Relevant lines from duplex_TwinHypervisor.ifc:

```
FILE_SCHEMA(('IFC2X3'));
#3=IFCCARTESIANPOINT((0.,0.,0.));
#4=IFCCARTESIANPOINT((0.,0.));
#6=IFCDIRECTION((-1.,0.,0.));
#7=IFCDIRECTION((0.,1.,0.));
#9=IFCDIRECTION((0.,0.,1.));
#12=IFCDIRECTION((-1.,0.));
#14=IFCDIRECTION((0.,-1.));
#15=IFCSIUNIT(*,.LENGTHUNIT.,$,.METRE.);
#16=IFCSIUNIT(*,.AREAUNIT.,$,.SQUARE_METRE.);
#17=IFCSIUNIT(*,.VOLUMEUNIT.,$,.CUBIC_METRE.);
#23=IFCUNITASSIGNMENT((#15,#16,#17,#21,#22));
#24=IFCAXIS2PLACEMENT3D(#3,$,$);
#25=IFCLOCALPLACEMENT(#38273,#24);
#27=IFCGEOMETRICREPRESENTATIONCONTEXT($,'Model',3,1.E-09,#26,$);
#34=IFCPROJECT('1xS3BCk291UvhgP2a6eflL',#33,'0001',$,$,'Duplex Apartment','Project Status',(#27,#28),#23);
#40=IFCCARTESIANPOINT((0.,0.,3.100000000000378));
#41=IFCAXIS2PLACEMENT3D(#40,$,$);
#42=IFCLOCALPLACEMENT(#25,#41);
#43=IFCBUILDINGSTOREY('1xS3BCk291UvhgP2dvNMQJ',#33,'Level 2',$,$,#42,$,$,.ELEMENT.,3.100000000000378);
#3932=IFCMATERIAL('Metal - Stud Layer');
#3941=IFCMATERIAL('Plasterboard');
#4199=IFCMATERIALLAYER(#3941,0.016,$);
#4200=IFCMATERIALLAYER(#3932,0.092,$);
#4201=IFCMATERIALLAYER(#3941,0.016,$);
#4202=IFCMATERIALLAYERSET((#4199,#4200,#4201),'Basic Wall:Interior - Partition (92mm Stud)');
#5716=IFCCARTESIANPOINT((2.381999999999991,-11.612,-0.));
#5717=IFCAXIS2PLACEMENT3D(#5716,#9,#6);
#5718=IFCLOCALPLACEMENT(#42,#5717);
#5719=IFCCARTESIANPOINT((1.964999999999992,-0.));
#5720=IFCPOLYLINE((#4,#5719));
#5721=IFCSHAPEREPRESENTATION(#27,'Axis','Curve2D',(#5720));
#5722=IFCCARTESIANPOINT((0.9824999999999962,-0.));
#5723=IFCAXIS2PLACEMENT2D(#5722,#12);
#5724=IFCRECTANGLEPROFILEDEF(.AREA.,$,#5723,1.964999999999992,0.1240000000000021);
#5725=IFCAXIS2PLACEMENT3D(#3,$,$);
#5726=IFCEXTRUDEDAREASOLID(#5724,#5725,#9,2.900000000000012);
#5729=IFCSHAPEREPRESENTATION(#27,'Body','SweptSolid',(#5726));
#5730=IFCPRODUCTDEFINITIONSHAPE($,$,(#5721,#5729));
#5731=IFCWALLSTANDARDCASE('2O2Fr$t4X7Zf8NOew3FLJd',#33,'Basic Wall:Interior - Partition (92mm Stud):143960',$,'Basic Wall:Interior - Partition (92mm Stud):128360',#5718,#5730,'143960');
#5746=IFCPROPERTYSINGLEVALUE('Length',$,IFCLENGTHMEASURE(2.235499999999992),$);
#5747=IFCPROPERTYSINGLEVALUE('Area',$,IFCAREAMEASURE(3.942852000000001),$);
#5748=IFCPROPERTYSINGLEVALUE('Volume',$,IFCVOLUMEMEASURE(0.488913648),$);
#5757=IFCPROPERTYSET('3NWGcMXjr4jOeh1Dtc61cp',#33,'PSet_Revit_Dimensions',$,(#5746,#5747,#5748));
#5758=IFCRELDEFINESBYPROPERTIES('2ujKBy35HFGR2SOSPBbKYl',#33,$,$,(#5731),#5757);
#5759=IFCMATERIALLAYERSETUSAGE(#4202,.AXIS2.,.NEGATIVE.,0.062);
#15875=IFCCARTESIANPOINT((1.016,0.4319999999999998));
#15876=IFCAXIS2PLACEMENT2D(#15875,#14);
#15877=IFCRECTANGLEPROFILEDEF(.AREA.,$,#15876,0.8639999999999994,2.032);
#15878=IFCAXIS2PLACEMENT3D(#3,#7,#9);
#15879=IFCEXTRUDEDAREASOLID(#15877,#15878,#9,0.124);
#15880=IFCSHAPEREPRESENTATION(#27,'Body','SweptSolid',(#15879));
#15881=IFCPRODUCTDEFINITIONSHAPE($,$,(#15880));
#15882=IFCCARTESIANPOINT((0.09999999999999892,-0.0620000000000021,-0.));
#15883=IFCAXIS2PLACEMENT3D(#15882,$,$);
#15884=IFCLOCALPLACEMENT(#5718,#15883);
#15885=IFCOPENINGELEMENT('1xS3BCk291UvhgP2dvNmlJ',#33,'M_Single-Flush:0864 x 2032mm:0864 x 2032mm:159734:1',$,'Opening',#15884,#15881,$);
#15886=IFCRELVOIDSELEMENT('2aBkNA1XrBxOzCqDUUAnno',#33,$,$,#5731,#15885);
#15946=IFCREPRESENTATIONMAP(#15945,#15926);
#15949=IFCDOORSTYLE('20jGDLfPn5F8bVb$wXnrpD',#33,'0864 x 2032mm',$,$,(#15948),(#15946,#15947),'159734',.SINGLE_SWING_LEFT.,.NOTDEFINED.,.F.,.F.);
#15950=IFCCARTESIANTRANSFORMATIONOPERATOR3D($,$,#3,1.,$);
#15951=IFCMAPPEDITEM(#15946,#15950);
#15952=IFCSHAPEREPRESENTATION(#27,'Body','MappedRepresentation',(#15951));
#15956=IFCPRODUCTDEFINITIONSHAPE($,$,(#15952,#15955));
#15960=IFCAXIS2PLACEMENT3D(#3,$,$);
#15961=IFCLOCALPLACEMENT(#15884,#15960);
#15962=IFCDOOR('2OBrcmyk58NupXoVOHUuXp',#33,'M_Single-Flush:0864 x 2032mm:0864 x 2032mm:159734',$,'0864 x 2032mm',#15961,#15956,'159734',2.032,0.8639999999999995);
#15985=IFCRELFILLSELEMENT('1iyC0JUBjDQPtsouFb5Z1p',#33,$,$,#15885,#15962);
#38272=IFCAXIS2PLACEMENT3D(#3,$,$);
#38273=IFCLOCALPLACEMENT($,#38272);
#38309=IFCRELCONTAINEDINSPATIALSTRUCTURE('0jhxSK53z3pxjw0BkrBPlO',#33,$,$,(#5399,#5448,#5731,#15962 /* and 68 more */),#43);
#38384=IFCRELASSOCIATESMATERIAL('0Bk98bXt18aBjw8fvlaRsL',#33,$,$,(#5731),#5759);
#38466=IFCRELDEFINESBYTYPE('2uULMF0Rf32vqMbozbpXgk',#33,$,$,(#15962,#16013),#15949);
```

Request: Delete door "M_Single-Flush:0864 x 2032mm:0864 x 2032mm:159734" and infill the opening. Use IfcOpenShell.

```python
import ifcopenshell
import ifcopenshell.api.feature
import ifcopenshell.api.pset
import ifcopenshell.api.root
import ifcopenshell.geom
import ifcopenshell.util.element
import ifcopenshell.util.shape
import ifcopenshell.util.unit

model = ifcopenshell.open("duplex_TwinHypervisor.ifc")
area_scale = ifcopenshell.util.unit.calculate_unit_scale(model, "AREAUNIT")
volume_scale = ifcopenshell.util.unit.calculate_unit_scale(model, "VOLUMEUNIT")
settings = ifcopenshell.geom.settings()


def volume(element):
    """Net volume in cubic metres, openings subtracted."""
    shape = ifcopenshell.geom.create_shape(settings, element)
    return ifcopenshell.util.shape.get_volume(shape.geometry)


door = model.by_guid("2OBrcmyk58NupXoVOHUuXp")
opening = door.FillsVoids[0].RelatingOpeningElement
wall = opening.VoidsElements[0].RelatingBuildingElement
before = volume(wall)

ifcopenshell.api.root.remove_product(model, product=door)
ifcopenshell.api.feature.remove_feature(model, feature=opening)

after = volume(wall)
thickness = 0.124  # wall thickness in metres

# Update the wall's stored quantities.
pset = model.by_id(ifcopenshell.util.element.get_pset(wall, "PSet_Revit_Dimensions", should_inherit=False)["id"])
ifcopenshell.api.pset.edit_pset(model, pset=pset, properties={
    "Area": model.create_entity("IfcAreaMeasure", after / thickness / area_scale),
    "Volume": model.create_entity("IfcVolumeMeasure", after / volume_scale),
})

print(f"wall volume {before:.3f} -> {after:.3f} m3")

model.write("duplex_TwinHypervisor_v2.ifc")
```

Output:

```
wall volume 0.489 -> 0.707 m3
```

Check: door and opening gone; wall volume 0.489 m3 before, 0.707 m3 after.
